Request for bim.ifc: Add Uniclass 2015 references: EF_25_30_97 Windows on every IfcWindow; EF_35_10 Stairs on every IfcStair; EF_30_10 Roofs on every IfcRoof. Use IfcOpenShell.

First a look at what the model holds.

```python
import ifcopenshell

model = ifcopenshell.open("bim.ifc")
print(model.schema)
print("classifications:", [c.Name for c in model.by_type("IfcClassification")])
for ifc_class in ("IfcDoor", "IfcRoof", "IfcStair", "IfcWall", "IfcWindow"):
    print(ifc_class, len(model.by_type(ifc_class)))
```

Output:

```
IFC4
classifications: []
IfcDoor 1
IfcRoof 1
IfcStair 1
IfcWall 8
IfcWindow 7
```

```python
import ifcopenshell
import ifcopenshell.api.classification

model = ifcopenshell.open("bim.ifc")

system = ifcopenshell.api.classification.add_classification(model, classification="Uniclass 2015")

codes = {
    "IfcWindow": ("EF_25_30_97", "Windows"),
    "IfcStair": ("EF_35_10", "Stairs"),
    "IfcRoof": ("EF_30_10", "Roofs"),
}
for ifc_class, (code, name) in codes.items():
    products = model.by_type(ifc_class)
    ifcopenshell.api.classification.add_reference(
        model, products=products, classification=system, identification=code, name=name
    )
    print(code, len(products))

model.write("bim_v2.ifc")
```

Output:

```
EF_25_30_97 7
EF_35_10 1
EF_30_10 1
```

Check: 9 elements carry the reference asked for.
